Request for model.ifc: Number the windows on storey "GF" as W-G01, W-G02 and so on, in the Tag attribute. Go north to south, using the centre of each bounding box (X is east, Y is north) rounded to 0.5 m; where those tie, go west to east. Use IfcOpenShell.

First a look at what the model holds.

```python
import ifcopenshell
import ifcopenshell.util.element
import ifcopenshell.util.placement

model = ifcopenshell.open("model.ifc")
print(model.schema)
storey = next(s for s in model.by_type("IfcBuildingStorey") if s.Name == "GF")
windows = [e for e in ifcopenshell.util.element.get_decomposition(storey) if e.is_a("IfcWindow")]
for e in sorted(windows, key=lambda e: e.id()):
    origin = ifcopenshell.util.placement.get_local_placement(e.ObjectPlacement)[:3, 3]
    print(e.id(), e.Tag, e.Name, origin.round(2) + 0.0, sep=" | ")
```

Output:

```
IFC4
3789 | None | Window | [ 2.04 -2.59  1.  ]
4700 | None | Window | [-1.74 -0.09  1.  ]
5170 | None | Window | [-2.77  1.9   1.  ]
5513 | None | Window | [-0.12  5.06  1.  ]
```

```python
import ifcopenshell
import ifcopenshell.geom
import ifcopenshell.util.element
import ifcopenshell.util.shape

model = ifcopenshell.open("model.ifc")
settings = ifcopenshell.geom.settings()
settings.set("use-world-coords", True)


def centre(element):
    shape = ifcopenshell.geom.create_shape(settings, element)
    return ifcopenshell.util.shape.get_bbox_centroid(shape.geometry)


storey = next(s for s in model.by_type("IfcBuildingStorey") if s.Name == "GF")
windows = [e for e in ifcopenshell.util.element.get_decomposition(storey) if e.is_a("IfcWindow")]

# Insertion points can sit at a corner or the storey origin, so sort by the geometry (in metres).
centres = {e: centre(e) for e in windows}
windows.sort(key=lambda e: (-round(centres[e][1] / 0.5), centres[e][0]))

for i, e in enumerate(windows, start=1):
    number = f"W-G{i:02d}"
    e.Tag = number
    print(e.id(), number)

model.write("model_rev.ifc")
```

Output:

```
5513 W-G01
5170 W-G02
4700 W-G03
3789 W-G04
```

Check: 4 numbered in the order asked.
